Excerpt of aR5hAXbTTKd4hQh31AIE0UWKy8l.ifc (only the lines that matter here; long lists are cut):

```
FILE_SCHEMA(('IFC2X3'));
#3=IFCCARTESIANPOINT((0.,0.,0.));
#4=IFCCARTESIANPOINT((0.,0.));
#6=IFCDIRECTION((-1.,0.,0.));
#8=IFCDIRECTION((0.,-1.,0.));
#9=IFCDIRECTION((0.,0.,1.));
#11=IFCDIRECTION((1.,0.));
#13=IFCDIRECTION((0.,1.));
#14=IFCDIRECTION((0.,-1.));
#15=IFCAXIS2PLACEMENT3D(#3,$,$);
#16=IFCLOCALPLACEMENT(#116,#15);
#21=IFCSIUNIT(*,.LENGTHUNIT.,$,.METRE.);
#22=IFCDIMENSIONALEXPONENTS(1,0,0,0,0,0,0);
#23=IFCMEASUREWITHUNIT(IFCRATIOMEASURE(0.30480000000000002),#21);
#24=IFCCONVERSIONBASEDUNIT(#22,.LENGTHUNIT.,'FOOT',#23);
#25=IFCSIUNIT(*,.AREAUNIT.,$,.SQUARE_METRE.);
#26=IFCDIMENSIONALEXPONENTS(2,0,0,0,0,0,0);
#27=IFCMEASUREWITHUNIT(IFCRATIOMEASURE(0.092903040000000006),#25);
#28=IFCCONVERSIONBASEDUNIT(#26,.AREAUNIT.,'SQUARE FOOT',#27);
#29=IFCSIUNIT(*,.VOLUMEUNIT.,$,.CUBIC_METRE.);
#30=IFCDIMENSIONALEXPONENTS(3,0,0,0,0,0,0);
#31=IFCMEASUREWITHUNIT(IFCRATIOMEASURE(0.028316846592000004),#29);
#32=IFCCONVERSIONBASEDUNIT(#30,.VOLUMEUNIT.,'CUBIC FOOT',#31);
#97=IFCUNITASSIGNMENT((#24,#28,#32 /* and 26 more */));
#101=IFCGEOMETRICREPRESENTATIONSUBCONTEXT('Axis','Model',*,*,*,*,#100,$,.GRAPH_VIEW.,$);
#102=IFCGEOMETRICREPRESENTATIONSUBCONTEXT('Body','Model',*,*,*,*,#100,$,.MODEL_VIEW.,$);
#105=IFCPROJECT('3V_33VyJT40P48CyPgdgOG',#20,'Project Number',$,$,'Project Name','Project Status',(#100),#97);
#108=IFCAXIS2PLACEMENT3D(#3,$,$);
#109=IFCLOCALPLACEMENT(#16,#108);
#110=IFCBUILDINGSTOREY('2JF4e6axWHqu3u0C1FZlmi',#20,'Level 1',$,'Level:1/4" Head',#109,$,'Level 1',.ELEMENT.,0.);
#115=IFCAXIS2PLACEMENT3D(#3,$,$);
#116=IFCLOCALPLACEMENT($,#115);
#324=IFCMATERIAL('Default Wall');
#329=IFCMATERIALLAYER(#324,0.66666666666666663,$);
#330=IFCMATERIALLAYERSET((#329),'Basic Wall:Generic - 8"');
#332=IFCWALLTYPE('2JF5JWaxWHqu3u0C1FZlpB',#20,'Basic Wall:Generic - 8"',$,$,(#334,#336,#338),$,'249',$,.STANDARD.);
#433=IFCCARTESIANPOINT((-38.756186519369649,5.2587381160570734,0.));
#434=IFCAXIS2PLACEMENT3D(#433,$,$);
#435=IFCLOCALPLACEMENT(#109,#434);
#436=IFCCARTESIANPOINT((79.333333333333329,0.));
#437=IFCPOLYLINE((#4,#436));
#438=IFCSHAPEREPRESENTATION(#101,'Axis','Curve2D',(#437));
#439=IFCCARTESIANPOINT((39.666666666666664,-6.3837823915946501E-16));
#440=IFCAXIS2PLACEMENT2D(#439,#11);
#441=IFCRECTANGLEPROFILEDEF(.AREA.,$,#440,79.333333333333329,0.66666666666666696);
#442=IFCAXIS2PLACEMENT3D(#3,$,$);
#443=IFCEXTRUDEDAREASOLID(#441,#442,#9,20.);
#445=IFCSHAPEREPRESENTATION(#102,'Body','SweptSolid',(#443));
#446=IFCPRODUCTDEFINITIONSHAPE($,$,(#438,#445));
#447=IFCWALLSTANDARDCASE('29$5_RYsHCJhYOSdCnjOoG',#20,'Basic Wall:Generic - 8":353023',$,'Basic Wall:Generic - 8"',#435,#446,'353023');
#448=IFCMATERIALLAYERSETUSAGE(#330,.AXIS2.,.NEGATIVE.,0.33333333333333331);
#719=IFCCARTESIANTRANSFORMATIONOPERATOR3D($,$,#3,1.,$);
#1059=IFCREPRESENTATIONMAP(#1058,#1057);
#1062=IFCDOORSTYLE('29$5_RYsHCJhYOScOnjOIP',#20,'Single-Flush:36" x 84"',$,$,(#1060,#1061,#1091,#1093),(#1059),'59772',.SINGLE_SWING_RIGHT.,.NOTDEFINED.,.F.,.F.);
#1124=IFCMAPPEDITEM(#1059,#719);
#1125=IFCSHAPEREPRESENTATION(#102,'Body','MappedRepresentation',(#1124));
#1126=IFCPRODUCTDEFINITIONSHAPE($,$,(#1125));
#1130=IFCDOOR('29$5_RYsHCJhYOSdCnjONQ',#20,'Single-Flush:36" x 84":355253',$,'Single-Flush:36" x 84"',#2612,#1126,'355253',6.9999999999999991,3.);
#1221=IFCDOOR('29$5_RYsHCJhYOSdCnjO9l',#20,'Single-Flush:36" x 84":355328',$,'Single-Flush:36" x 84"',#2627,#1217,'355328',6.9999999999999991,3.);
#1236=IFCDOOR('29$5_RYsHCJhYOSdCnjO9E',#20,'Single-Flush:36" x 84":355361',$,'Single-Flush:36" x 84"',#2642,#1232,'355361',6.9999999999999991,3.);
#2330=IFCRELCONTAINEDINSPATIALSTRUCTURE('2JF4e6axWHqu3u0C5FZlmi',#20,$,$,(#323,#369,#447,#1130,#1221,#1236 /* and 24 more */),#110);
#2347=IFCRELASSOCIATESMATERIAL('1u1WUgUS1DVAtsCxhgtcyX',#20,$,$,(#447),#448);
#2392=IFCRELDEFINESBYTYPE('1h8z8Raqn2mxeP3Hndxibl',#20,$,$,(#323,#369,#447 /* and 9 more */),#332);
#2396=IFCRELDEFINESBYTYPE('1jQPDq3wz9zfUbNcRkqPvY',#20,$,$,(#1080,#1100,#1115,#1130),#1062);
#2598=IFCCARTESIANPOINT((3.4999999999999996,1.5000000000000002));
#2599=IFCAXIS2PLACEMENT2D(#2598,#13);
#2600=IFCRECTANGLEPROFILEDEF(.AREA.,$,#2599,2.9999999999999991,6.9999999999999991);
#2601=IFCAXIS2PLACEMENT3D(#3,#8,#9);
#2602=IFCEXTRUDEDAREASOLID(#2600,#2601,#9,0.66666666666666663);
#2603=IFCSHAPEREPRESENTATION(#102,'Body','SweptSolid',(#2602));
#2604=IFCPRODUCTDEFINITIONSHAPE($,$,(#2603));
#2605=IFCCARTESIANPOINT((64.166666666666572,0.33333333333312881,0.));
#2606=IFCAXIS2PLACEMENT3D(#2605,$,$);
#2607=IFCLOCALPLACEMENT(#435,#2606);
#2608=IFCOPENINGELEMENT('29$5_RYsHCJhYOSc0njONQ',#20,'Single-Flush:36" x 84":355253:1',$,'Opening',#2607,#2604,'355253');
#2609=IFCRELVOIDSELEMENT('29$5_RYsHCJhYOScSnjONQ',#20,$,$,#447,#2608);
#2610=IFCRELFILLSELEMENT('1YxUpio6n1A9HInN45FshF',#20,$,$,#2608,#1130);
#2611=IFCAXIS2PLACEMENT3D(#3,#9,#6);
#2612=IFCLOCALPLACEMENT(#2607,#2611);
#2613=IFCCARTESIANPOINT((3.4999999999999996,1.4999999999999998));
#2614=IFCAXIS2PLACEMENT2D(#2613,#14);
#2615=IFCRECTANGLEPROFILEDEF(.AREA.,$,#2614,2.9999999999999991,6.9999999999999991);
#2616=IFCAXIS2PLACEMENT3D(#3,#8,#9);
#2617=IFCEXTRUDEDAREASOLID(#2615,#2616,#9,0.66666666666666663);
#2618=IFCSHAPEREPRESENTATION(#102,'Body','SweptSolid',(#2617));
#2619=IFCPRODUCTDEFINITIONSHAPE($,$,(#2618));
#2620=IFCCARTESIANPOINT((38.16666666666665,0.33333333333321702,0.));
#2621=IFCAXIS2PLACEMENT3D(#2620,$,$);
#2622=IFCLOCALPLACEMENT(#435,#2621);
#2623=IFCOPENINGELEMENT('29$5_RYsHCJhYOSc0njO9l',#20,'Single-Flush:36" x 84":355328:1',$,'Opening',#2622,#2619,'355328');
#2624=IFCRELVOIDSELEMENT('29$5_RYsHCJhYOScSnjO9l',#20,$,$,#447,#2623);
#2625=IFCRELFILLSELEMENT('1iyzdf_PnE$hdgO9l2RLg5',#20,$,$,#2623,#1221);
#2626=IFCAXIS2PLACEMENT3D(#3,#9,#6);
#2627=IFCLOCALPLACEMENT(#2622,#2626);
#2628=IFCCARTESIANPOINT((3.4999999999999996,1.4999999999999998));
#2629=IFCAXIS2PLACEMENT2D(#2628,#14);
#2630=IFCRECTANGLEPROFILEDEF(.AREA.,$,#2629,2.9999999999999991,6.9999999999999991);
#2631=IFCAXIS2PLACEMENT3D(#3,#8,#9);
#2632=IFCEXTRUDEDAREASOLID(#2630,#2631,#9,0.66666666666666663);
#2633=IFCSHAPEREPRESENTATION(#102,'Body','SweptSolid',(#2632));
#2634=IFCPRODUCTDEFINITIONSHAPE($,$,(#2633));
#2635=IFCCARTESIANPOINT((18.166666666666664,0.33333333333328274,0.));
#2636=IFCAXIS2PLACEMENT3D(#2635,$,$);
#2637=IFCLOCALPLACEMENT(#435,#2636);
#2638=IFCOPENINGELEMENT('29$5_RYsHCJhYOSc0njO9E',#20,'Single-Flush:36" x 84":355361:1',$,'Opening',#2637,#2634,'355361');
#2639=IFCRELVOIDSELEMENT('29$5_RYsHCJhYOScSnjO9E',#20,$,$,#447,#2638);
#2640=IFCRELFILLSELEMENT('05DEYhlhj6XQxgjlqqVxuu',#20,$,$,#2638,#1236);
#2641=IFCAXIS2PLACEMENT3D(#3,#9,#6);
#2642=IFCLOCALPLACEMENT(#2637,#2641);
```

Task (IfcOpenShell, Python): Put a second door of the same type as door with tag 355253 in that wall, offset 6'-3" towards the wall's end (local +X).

```python
import ifcopenshell
import ifcopenshell.api.feature
import ifcopenshell.api.geometry
import ifcopenshell.api.root
import ifcopenshell.geom
import ifcopenshell.util.element
import ifcopenshell.util.placement
import ifcopenshell.util.shape
import ifcopenshell.util.unit

model = ifcopenshell.open("aR5hAXbTTKd4hQh31AIE0UWKy8l.ifc")
unit_scale = ifcopenshell.util.unit.calculate_unit_scale(model)
settings = ifcopenshell.geom.settings()


def volume(element):
    """Net volume in cubic metres, openings subtracted."""
    shape = ifcopenshell.geom.create_shape(settings, element)
    return ifcopenshell.util.shape.get_volume(shape.geometry)


def reuse_history(source, copy):
    """copy_class also copies each property set's owner history, people and application; keep the originals."""
    for rel in copy.IsDefinedBy:
        if rel.is_a("IfcRelDefinesByProperties") and (history := rel.RelatingPropertyDefinition.OwnerHistory):
            rel.RelatingPropertyDefinition.OwnerHistory = source.OwnerHistory
            ifcopenshell.util.element.remove_deep2(model, history)


door = model.by_guid("29$5_RYsHCJhYOSdCnjONQ")
opening = door.FillsVoids[0].RelatingOpeningElement
wall = opening.VoidsElements[0].RelatingBuildingElement
before = volume(wall)
shift = ifcopenshell.util.placement.get_local_placement(wall.ObjectPlacement)[:3, 0] * 75 * 0.0254 / unit_scale

# copy_class copies the void relationship, type, container and properties, but no geometry.
new_opening = ifcopenshell.api.root.copy_class(model, product=opening)
new_opening.Representation = ifcopenshell.util.element.copy_deep(
    model, opening.Representation, exclude=["IfcGeometricRepresentationContext", "IfcRepresentationMap"]
)
new_opening.Name = 'Single-Flush:36" x 84"'
new_opening.Tag = None
new_door = ifcopenshell.api.root.copy_class(model, product=door)
new_door.Representation = ifcopenshell.util.element.copy_deep(
    model, door.Representation, exclude=["IfcGeometricRepresentationContext", "IfcRepresentationMap"]
)
new_door.Name = 'Single-Flush:36" x 84"'
new_door.Tag = None
reuse_history(door, new_door)
fills = ifcopenshell.api.feature.add_filling(model, opening=new_opening, element=new_door)
fills.OwnerHistory = new_door.OwnerHistory  # required in IFC2X3

for old, new in ((opening, new_opening), (door, new_door)):
    matrix = ifcopenshell.util.placement.get_local_placement(old.ObjectPlacement)
    matrix[:3, 3] += shift
    ifcopenshell.api.geometry.edit_object_placement(model, product=new, matrix=matrix, is_si=False)

after = volume(wall)

print(f"wall volume {before:.3f} -> {after:.3f} m3")

model.write("aR5hAXbTTKd4hQh31AIE0UWKy8l_updated.ifc")
```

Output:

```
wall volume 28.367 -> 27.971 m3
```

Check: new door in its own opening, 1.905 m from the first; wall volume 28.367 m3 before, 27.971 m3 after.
